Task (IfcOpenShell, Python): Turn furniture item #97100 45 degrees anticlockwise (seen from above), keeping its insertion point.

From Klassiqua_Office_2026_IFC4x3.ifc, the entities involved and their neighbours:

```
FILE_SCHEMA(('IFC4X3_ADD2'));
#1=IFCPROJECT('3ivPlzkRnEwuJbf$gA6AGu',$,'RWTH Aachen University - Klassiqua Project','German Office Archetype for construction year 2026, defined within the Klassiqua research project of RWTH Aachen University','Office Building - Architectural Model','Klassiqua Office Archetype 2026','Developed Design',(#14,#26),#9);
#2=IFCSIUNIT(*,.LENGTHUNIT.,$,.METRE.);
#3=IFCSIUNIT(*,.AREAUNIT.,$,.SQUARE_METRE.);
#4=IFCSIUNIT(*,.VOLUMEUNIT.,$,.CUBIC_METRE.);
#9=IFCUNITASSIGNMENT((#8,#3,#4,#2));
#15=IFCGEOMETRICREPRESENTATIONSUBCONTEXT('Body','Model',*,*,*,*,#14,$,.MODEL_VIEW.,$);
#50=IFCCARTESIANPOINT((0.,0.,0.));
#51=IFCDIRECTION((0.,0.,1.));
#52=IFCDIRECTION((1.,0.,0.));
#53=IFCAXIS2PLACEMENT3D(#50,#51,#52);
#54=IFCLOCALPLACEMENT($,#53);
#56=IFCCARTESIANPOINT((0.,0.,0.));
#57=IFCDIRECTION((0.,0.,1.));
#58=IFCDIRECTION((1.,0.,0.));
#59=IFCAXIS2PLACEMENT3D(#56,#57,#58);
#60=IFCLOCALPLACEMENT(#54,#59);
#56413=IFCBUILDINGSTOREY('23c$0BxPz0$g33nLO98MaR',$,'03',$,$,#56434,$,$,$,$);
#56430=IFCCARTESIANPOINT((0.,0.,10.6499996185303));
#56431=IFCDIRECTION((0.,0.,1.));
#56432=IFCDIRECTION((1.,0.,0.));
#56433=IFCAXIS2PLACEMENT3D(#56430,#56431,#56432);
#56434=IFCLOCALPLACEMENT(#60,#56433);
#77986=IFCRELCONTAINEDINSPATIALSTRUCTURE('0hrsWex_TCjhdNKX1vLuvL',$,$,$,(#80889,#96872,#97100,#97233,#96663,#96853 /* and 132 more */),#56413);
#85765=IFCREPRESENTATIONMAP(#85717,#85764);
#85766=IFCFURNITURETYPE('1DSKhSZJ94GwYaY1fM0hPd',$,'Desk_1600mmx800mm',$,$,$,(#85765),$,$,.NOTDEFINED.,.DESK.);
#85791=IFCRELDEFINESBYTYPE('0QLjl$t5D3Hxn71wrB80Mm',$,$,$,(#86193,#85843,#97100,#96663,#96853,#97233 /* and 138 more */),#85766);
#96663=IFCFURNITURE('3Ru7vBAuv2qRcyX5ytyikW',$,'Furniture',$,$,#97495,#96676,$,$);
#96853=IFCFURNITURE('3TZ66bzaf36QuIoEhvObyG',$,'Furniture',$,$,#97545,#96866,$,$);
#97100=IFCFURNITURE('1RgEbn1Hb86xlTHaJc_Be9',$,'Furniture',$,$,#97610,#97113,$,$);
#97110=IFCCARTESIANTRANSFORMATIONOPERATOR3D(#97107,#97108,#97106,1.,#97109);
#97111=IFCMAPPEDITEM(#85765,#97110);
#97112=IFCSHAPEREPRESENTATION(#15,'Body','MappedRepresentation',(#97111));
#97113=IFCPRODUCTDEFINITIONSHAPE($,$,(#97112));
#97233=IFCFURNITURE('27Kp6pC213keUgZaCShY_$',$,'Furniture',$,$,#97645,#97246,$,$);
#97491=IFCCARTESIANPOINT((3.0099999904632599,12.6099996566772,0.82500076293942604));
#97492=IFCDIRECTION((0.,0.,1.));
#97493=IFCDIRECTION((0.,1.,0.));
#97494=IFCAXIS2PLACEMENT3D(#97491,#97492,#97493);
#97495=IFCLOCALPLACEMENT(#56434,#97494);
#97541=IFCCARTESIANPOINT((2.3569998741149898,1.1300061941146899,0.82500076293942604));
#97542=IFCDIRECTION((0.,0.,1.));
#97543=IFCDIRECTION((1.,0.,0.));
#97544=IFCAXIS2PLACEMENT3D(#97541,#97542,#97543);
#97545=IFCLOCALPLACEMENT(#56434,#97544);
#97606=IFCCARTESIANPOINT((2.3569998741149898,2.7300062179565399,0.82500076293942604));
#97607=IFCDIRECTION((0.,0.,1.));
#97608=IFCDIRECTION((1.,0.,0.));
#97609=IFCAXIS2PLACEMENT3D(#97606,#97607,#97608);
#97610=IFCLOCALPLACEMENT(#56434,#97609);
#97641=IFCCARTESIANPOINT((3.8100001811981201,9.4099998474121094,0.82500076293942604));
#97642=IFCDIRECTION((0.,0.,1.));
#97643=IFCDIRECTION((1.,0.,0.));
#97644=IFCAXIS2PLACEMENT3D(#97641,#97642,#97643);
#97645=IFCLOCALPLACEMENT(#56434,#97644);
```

```python
import ifcopenshell
import ifcopenshell.api.geometry
import ifcopenshell.util.placement

model = ifcopenshell.open("Klassiqua_Office_2026_IFC4x3.ifc")

item = model.by_id(97100)
matrix = ifcopenshell.util.placement.get_local_placement(item.ObjectPlacement)
matrix = matrix @ ifcopenshell.util.placement.rotation(45, "Z")
ifcopenshell.api.geometry.edit_object_placement(model, product=item, matrix=matrix, is_si=False)

print(ifcopenshell.util.placement.get_local_placement(item.ObjectPlacement).round(3) + 0.0)

model.write("Klassiqua_Office_2026_IFC4x3_rev.ifc")
```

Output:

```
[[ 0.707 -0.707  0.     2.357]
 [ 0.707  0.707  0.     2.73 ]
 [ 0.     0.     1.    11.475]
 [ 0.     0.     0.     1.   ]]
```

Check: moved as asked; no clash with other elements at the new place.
